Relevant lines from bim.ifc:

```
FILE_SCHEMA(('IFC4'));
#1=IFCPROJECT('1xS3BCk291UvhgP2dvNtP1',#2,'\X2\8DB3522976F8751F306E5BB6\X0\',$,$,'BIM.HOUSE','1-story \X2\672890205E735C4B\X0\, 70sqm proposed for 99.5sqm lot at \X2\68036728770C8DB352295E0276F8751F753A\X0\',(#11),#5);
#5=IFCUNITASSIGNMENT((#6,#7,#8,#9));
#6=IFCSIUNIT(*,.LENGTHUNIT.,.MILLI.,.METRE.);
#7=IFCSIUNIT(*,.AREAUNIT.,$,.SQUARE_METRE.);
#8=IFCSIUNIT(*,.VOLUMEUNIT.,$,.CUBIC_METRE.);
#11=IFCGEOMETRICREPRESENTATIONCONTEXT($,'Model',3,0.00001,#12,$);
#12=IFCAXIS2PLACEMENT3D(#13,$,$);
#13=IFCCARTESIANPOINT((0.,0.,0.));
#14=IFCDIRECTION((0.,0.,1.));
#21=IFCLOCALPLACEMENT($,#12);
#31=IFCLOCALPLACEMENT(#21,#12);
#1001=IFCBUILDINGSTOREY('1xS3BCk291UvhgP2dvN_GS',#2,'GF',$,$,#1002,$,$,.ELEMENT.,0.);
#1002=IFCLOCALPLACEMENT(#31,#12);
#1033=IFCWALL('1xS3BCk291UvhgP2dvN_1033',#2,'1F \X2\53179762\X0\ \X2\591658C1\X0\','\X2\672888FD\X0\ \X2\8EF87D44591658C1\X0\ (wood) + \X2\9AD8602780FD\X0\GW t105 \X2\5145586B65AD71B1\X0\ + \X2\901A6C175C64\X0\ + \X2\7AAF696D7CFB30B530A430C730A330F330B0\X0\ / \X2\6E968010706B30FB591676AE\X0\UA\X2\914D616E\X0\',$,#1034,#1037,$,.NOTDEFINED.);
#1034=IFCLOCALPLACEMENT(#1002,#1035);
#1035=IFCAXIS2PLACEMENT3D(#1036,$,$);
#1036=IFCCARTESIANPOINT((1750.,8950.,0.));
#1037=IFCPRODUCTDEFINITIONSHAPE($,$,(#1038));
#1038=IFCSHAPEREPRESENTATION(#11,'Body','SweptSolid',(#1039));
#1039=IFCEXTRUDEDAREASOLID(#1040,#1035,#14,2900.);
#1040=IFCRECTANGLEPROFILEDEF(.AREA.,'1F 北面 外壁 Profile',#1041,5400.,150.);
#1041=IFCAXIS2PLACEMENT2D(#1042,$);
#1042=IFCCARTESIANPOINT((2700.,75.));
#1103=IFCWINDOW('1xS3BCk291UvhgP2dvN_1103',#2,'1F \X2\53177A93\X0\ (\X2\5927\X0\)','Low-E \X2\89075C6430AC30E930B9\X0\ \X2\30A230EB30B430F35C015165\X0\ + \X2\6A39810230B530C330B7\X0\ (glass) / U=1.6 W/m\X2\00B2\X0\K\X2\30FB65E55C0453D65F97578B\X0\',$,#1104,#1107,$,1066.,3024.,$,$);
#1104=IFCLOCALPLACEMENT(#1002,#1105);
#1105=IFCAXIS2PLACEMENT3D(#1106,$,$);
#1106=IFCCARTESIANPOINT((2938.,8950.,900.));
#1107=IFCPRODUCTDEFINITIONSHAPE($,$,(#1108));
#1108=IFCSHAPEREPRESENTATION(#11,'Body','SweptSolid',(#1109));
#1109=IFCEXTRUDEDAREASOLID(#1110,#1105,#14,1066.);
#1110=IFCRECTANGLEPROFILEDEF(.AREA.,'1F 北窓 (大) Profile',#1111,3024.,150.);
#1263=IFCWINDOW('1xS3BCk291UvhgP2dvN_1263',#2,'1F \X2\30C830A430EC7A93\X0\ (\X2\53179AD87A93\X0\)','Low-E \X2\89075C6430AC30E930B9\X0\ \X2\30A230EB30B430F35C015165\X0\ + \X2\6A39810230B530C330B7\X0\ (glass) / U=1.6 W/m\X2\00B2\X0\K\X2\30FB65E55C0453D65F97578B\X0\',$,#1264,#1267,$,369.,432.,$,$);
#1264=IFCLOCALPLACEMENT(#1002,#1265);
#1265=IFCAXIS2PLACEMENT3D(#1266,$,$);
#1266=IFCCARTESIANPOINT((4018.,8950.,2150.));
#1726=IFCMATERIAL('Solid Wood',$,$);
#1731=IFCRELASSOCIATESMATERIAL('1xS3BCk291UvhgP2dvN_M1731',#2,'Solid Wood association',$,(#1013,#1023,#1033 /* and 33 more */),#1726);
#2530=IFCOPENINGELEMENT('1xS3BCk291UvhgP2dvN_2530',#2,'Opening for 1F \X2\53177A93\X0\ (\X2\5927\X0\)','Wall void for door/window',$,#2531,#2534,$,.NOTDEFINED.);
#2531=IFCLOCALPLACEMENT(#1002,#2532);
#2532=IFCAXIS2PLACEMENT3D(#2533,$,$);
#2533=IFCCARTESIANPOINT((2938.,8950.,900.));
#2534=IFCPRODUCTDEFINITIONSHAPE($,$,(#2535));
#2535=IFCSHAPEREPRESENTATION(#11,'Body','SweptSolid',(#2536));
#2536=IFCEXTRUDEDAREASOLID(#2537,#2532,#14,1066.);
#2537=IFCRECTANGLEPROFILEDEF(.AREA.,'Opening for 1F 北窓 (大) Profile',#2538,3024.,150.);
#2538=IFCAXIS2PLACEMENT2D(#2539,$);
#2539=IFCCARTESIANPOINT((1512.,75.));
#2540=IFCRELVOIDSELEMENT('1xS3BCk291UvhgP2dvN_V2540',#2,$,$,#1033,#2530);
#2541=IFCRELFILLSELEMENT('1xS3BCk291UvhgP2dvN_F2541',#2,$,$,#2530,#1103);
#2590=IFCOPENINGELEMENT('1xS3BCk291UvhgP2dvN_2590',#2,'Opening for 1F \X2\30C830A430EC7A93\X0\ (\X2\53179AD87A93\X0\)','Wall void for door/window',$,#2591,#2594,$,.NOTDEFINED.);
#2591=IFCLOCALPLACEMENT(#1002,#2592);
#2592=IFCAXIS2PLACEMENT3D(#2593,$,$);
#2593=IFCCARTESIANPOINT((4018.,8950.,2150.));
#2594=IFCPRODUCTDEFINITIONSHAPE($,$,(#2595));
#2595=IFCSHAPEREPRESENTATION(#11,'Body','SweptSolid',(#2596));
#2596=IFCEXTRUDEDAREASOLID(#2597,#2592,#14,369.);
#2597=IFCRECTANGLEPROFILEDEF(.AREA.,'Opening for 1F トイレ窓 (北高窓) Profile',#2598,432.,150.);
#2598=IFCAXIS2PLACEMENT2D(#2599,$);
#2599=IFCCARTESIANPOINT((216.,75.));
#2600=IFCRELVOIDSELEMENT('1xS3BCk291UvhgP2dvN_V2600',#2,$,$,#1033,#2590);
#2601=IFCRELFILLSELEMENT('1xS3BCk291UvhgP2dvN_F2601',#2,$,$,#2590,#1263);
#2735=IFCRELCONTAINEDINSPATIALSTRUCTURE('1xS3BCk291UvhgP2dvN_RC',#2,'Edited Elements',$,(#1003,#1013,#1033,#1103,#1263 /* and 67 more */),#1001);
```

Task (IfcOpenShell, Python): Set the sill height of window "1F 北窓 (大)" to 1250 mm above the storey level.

```python
import numpy as np
import ifcopenshell
import ifcopenshell.api.geometry
import ifcopenshell.geom
import ifcopenshell.util.element
import ifcopenshell.util.placement
import ifcopenshell.util.shape
import ifcopenshell.util.unit

model = ifcopenshell.open("bim.ifc")
unit_scale = ifcopenshell.util.unit.calculate_unit_scale(model)

window = model.by_guid("1xS3BCk291UvhgP2dvN_1103")
opening = window.FillsVoids[0].RelatingOpeningElement
storey = ifcopenshell.util.element.get_container(window, ifc_class="IfcBuildingStorey")
level = ifcopenshell.util.placement.get_local_placement(storey.ObjectPlacement)[2, 3]

# The opening's origin need not be at the sill, so measure its lowest point.
shape = ifcopenshell.geom.create_shape(ifcopenshell.geom.settings(), opening)
bottom = ifcopenshell.util.shape.get_shape_bottom_elevation(shape, shape.geometry) / unit_scale
dz = level + 1250.0 - bottom

shift = np.array([0.0, 0.0, dz])
# The window is not placed relative to its opening, so move both.
for product in (opening, window):
    matrix = ifcopenshell.util.placement.get_local_placement(product.ObjectPlacement)
    matrix[:3, 3] += shift
    ifcopenshell.api.geometry.edit_object_placement(model, product=product, matrix=matrix, is_si=False)

print(f"moved by {dz * unit_scale:+.3f} m")

model.write("bim_v2.ifc")
```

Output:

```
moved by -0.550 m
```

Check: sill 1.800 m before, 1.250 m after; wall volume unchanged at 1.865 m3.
